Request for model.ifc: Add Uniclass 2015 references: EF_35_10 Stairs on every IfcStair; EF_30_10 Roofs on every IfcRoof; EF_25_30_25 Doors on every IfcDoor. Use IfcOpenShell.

First a look at what the model holds.

```python
import ifcopenshell

model = ifcopenshell.open("model.ifc")
print(model.schema)
print("classifications:", [c.Name for c in model.by_type("IfcClassification")])
for ifc_class in ("IfcDoor", "IfcRoof", "IfcStair", "IfcWall", "IfcWindow"):
    print(ifc_class, len(model.by_type(ifc_class)))
```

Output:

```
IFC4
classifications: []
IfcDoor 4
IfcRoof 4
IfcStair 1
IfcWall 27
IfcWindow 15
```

```python
import ifcopenshell
import ifcopenshell.api.classification

model = ifcopenshell.open("model.ifc")

system = ifcopenshell.api.classification.add_classification(model, classification="Uniclass 2015")

codes = {
    "IfcStair": ("EF_35_10", "Stairs"),
    "IfcRoof": ("EF_30_10", "Roofs"),
    "IfcDoor": ("EF_25_30_25", "Doors"),
}
for ifc_class, (code, name) in codes.items():
    products = model.by_type(ifc_class)
    ifcopenshell.api.classification.add_reference(
        model, products=products, classification=system, identification=code, name=name
    )
    print(code, len(products))

model.write("model-out.ifc")
```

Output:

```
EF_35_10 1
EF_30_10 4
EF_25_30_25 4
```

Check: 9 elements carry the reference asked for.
